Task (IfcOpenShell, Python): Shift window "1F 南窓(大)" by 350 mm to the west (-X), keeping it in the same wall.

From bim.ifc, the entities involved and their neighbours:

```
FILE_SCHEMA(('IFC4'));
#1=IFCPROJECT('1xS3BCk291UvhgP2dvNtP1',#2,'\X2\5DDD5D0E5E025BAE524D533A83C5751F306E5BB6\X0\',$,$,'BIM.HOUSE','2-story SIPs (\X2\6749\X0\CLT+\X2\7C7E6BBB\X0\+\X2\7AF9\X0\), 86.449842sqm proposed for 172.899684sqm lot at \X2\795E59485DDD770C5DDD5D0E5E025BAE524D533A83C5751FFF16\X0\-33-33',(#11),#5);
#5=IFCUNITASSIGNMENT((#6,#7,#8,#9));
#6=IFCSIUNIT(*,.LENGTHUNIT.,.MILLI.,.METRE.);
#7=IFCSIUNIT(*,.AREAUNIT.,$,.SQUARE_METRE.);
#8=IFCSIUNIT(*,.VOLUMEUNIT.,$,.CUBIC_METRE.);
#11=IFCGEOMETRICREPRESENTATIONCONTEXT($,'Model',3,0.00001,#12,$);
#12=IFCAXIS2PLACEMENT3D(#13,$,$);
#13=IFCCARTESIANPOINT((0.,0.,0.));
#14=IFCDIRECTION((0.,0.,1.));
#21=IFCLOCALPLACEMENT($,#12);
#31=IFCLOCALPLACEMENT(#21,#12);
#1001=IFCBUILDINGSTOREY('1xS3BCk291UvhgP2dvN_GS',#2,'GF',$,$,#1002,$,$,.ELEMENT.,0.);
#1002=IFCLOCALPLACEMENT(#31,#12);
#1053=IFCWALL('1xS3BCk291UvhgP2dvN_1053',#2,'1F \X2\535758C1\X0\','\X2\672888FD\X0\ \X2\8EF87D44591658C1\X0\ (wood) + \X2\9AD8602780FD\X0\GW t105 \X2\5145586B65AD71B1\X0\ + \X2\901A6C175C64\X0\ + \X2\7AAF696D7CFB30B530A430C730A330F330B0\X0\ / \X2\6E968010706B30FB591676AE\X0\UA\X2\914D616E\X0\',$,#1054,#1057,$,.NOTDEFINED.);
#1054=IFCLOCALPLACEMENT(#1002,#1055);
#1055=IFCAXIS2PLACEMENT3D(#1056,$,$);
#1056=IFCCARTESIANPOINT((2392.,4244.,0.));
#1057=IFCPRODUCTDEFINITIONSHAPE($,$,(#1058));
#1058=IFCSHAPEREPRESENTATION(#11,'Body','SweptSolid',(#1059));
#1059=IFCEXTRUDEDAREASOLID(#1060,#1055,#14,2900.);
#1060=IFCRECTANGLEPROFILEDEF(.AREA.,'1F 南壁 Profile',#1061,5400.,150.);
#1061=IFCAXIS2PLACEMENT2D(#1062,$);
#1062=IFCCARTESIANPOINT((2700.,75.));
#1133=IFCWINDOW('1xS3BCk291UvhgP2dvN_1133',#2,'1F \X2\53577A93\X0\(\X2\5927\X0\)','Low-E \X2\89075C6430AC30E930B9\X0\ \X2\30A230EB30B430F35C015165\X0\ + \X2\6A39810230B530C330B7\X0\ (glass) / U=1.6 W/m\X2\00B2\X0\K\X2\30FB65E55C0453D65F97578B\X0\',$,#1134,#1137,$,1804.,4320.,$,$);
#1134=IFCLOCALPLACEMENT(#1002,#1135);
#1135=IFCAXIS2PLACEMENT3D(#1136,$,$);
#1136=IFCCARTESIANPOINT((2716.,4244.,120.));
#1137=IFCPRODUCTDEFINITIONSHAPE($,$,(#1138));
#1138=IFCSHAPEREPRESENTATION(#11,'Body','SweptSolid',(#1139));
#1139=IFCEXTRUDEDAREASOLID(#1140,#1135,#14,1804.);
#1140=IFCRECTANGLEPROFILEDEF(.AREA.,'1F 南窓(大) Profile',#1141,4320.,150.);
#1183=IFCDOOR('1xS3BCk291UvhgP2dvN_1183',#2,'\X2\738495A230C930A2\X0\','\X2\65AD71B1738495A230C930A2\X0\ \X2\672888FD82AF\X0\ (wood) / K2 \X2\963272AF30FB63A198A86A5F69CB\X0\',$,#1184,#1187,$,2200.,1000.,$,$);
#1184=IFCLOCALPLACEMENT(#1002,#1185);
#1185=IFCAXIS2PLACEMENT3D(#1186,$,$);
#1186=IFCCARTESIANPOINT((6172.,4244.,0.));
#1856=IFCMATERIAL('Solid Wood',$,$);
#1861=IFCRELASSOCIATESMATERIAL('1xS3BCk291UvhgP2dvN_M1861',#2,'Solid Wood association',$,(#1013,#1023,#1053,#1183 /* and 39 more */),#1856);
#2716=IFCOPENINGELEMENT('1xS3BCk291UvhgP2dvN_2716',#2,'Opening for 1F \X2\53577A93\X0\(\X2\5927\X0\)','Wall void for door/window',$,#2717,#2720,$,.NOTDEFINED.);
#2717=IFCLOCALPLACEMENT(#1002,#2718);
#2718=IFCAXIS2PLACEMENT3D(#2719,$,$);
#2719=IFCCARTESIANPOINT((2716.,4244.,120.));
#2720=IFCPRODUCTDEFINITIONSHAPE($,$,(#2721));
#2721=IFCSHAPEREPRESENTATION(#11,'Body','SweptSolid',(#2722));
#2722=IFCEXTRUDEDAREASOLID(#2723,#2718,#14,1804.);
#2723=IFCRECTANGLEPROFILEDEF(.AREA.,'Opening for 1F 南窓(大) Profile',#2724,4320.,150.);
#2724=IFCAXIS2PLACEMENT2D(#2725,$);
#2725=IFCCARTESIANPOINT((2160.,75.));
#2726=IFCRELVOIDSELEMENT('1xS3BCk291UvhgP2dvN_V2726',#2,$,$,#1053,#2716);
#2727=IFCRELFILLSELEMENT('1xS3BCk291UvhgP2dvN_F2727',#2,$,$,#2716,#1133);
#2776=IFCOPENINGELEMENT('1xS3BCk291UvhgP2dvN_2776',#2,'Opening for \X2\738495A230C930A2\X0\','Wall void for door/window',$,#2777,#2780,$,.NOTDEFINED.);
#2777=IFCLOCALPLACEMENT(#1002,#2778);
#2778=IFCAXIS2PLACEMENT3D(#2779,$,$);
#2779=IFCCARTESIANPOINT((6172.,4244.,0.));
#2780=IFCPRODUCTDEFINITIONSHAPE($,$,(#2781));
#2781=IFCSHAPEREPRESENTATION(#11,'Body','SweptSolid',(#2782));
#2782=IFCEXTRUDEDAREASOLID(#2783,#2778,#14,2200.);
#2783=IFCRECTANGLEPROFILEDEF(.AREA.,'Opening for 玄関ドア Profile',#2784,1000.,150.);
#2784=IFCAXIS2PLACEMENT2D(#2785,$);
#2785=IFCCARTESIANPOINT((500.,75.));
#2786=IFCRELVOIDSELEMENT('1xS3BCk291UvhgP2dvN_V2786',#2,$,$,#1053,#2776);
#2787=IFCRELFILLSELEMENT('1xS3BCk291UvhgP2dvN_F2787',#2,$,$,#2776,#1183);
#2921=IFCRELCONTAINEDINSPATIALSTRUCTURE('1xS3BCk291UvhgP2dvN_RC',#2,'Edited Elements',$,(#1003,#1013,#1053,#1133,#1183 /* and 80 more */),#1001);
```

```python
import ifcopenshell
import ifcopenshell.api.geometry
import ifcopenshell.util.placement
import ifcopenshell.util.unit

model = ifcopenshell.open("bim.ifc")
unit_scale = ifcopenshell.util.unit.calculate_unit_scale(model)

window = model.by_id(1133)
opening = window.FillsVoids[0].RelatingOpeningElement
wall = opening.VoidsElements[0].RelatingBuildingElement

wall_matrix = ifcopenshell.util.placement.get_local_placement(wall.ObjectPlacement)
shift = wall_matrix[:3, 0] * -0.35 / unit_scale
before = ifcopenshell.util.placement.get_local_placement(window.ObjectPlacement)[:3, 3].copy()

# The window is not placed relative to its opening, so move both.
for product in (opening, window):
    matrix = ifcopenshell.util.placement.get_local_placement(product.ObjectPlacement)
    matrix[:3, 3] += shift
    ifcopenshell.api.geometry.edit_object_placement(model, product=product, matrix=matrix, is_si=False)

after = ifcopenshell.util.placement.get_local_placement(window.ObjectPlacement)[:3, 3]
print("window moved by", (after - before).round(3) + 0.0)

model.write("bim-out.ifc")
```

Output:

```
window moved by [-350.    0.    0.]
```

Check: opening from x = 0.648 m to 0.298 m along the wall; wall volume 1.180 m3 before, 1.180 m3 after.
